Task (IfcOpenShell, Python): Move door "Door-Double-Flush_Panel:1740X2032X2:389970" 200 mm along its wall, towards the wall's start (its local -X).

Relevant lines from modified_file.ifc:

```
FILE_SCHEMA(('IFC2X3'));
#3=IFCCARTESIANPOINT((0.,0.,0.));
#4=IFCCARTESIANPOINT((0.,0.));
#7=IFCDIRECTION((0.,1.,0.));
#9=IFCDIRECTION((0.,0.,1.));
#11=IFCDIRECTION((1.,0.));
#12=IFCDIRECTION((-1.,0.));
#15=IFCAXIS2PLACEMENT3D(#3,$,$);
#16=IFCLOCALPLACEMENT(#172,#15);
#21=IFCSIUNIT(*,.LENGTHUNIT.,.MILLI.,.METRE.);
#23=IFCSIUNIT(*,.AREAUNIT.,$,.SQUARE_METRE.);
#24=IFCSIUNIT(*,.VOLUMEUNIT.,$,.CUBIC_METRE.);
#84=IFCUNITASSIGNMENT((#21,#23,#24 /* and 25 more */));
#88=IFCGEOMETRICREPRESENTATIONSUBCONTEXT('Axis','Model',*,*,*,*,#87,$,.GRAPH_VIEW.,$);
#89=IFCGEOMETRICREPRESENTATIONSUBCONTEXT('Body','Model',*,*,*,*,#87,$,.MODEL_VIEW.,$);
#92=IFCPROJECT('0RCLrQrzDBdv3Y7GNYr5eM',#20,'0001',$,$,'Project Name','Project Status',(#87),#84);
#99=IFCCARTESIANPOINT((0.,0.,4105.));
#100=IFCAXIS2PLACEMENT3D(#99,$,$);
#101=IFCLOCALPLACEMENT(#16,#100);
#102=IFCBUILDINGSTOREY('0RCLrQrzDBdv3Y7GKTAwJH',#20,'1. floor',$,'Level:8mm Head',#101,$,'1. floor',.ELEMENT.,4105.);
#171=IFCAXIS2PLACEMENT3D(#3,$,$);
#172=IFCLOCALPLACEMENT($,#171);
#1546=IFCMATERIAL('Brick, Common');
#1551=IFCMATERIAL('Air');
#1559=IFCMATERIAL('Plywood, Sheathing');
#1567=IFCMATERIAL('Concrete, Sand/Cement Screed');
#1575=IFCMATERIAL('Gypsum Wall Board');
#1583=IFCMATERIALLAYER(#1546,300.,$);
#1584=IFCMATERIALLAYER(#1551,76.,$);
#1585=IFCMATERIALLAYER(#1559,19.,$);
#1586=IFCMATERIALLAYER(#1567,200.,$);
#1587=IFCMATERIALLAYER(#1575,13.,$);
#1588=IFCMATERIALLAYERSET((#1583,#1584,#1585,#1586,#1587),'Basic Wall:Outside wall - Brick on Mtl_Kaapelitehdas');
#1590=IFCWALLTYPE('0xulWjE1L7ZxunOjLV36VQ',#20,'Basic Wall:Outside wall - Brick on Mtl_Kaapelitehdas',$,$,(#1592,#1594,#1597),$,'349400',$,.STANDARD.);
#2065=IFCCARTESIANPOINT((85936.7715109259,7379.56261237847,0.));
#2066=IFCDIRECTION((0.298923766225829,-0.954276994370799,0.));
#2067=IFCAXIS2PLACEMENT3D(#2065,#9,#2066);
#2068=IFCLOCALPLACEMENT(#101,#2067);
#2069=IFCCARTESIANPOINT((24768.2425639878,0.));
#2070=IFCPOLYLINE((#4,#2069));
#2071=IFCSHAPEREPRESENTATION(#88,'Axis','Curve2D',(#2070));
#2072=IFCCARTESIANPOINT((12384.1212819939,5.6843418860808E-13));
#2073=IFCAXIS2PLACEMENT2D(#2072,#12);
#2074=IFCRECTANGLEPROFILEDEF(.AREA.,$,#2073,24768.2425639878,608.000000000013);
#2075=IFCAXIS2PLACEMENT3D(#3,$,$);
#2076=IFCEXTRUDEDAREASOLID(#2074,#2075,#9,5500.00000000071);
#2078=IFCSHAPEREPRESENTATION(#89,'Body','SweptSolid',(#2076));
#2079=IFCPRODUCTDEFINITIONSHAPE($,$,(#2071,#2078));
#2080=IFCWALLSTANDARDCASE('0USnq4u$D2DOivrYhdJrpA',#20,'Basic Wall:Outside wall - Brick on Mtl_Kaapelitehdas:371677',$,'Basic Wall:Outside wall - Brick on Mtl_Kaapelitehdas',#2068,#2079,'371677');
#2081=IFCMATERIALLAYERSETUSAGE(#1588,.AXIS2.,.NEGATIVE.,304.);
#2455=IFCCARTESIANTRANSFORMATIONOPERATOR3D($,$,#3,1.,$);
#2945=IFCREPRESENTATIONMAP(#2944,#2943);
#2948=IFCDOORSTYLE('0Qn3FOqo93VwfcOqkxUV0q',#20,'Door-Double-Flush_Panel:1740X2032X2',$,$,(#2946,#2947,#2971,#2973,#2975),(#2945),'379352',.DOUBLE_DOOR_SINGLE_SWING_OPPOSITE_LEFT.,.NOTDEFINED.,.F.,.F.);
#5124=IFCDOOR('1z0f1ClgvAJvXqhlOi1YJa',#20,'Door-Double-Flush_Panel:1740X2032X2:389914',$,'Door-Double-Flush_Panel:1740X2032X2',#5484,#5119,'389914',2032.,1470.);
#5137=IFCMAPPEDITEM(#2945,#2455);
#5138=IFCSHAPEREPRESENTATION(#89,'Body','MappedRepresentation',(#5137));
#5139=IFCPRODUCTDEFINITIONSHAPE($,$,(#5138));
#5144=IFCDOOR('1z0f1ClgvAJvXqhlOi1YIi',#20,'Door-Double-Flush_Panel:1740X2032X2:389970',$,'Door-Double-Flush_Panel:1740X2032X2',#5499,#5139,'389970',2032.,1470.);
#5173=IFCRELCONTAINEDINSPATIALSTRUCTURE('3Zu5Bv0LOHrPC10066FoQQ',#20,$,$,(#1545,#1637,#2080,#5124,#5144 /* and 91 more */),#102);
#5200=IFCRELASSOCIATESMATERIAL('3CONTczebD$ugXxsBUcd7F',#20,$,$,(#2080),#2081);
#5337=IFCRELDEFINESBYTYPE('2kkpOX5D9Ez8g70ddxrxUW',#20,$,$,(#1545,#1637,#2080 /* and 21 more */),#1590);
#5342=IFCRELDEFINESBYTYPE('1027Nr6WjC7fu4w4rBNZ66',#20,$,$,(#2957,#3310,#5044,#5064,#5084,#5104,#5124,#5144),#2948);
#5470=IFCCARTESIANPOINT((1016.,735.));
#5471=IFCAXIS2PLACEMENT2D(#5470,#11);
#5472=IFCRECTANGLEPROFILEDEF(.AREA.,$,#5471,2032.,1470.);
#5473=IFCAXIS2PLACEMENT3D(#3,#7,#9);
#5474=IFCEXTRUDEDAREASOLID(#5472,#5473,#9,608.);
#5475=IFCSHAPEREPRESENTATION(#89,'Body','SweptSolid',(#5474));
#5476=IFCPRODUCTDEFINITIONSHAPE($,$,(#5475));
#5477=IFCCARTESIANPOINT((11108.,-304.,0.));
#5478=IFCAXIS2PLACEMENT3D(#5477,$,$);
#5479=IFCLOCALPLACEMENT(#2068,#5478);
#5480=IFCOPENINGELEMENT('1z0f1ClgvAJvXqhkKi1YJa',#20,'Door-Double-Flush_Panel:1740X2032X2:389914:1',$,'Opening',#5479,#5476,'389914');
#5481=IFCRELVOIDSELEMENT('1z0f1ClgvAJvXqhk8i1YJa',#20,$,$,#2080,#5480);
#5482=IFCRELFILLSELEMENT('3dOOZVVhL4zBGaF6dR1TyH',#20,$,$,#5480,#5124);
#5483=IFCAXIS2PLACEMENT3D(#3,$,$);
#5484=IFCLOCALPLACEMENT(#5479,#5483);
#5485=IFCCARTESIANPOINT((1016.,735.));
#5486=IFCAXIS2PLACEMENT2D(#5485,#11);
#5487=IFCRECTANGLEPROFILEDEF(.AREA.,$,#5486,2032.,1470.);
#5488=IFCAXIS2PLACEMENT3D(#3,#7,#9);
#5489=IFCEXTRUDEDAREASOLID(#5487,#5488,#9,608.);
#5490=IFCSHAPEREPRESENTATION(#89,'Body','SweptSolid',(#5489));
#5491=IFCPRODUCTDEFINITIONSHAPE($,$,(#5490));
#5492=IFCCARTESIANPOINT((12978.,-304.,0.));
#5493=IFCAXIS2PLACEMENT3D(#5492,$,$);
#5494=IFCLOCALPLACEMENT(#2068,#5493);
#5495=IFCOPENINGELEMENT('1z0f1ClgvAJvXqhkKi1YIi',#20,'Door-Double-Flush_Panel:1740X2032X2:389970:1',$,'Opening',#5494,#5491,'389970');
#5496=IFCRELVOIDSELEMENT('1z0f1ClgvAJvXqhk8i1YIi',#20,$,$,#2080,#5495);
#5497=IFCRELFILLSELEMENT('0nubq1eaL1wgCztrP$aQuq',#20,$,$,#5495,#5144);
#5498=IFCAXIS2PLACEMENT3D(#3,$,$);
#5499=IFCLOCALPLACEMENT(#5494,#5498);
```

```python
import ifcopenshell
import ifcopenshell.api.geometry
import ifcopenshell.util.placement

model = ifcopenshell.open("modified_file.ifc")

door = model.by_guid("1z0f1ClgvAJvXqhlOi1YIi")
opening = door.FillsVoids[0].RelatingOpeningElement
wall = opening.VoidsElements[0].RelatingBuildingElement

wall_matrix = ifcopenshell.util.placement.get_local_placement(wall.ObjectPlacement)
shift = wall_matrix[:3, 0] * -200.0
before = ifcopenshell.util.placement.get_local_placement(door.ObjectPlacement)[:3, 3].copy()

# The door is placed relative to its opening, so it follows when the opening moves.
matrix = ifcopenshell.util.placement.get_local_placement(opening.ObjectPlacement)
matrix[:3, 3] += shift
ifcopenshell.api.geometry.edit_object_placement(
    model, product=opening, matrix=matrix, is_si=False, should_transform_children=True
)

after = ifcopenshell.util.placement.get_local_placement(door.ObjectPlacement)[:3, 3]
print("door moved by", (after - before).round(3) + 0.0)

model.write("modified_file_updated.ifc")
```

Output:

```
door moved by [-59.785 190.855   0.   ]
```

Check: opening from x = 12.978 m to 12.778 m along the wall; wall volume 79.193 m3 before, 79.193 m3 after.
